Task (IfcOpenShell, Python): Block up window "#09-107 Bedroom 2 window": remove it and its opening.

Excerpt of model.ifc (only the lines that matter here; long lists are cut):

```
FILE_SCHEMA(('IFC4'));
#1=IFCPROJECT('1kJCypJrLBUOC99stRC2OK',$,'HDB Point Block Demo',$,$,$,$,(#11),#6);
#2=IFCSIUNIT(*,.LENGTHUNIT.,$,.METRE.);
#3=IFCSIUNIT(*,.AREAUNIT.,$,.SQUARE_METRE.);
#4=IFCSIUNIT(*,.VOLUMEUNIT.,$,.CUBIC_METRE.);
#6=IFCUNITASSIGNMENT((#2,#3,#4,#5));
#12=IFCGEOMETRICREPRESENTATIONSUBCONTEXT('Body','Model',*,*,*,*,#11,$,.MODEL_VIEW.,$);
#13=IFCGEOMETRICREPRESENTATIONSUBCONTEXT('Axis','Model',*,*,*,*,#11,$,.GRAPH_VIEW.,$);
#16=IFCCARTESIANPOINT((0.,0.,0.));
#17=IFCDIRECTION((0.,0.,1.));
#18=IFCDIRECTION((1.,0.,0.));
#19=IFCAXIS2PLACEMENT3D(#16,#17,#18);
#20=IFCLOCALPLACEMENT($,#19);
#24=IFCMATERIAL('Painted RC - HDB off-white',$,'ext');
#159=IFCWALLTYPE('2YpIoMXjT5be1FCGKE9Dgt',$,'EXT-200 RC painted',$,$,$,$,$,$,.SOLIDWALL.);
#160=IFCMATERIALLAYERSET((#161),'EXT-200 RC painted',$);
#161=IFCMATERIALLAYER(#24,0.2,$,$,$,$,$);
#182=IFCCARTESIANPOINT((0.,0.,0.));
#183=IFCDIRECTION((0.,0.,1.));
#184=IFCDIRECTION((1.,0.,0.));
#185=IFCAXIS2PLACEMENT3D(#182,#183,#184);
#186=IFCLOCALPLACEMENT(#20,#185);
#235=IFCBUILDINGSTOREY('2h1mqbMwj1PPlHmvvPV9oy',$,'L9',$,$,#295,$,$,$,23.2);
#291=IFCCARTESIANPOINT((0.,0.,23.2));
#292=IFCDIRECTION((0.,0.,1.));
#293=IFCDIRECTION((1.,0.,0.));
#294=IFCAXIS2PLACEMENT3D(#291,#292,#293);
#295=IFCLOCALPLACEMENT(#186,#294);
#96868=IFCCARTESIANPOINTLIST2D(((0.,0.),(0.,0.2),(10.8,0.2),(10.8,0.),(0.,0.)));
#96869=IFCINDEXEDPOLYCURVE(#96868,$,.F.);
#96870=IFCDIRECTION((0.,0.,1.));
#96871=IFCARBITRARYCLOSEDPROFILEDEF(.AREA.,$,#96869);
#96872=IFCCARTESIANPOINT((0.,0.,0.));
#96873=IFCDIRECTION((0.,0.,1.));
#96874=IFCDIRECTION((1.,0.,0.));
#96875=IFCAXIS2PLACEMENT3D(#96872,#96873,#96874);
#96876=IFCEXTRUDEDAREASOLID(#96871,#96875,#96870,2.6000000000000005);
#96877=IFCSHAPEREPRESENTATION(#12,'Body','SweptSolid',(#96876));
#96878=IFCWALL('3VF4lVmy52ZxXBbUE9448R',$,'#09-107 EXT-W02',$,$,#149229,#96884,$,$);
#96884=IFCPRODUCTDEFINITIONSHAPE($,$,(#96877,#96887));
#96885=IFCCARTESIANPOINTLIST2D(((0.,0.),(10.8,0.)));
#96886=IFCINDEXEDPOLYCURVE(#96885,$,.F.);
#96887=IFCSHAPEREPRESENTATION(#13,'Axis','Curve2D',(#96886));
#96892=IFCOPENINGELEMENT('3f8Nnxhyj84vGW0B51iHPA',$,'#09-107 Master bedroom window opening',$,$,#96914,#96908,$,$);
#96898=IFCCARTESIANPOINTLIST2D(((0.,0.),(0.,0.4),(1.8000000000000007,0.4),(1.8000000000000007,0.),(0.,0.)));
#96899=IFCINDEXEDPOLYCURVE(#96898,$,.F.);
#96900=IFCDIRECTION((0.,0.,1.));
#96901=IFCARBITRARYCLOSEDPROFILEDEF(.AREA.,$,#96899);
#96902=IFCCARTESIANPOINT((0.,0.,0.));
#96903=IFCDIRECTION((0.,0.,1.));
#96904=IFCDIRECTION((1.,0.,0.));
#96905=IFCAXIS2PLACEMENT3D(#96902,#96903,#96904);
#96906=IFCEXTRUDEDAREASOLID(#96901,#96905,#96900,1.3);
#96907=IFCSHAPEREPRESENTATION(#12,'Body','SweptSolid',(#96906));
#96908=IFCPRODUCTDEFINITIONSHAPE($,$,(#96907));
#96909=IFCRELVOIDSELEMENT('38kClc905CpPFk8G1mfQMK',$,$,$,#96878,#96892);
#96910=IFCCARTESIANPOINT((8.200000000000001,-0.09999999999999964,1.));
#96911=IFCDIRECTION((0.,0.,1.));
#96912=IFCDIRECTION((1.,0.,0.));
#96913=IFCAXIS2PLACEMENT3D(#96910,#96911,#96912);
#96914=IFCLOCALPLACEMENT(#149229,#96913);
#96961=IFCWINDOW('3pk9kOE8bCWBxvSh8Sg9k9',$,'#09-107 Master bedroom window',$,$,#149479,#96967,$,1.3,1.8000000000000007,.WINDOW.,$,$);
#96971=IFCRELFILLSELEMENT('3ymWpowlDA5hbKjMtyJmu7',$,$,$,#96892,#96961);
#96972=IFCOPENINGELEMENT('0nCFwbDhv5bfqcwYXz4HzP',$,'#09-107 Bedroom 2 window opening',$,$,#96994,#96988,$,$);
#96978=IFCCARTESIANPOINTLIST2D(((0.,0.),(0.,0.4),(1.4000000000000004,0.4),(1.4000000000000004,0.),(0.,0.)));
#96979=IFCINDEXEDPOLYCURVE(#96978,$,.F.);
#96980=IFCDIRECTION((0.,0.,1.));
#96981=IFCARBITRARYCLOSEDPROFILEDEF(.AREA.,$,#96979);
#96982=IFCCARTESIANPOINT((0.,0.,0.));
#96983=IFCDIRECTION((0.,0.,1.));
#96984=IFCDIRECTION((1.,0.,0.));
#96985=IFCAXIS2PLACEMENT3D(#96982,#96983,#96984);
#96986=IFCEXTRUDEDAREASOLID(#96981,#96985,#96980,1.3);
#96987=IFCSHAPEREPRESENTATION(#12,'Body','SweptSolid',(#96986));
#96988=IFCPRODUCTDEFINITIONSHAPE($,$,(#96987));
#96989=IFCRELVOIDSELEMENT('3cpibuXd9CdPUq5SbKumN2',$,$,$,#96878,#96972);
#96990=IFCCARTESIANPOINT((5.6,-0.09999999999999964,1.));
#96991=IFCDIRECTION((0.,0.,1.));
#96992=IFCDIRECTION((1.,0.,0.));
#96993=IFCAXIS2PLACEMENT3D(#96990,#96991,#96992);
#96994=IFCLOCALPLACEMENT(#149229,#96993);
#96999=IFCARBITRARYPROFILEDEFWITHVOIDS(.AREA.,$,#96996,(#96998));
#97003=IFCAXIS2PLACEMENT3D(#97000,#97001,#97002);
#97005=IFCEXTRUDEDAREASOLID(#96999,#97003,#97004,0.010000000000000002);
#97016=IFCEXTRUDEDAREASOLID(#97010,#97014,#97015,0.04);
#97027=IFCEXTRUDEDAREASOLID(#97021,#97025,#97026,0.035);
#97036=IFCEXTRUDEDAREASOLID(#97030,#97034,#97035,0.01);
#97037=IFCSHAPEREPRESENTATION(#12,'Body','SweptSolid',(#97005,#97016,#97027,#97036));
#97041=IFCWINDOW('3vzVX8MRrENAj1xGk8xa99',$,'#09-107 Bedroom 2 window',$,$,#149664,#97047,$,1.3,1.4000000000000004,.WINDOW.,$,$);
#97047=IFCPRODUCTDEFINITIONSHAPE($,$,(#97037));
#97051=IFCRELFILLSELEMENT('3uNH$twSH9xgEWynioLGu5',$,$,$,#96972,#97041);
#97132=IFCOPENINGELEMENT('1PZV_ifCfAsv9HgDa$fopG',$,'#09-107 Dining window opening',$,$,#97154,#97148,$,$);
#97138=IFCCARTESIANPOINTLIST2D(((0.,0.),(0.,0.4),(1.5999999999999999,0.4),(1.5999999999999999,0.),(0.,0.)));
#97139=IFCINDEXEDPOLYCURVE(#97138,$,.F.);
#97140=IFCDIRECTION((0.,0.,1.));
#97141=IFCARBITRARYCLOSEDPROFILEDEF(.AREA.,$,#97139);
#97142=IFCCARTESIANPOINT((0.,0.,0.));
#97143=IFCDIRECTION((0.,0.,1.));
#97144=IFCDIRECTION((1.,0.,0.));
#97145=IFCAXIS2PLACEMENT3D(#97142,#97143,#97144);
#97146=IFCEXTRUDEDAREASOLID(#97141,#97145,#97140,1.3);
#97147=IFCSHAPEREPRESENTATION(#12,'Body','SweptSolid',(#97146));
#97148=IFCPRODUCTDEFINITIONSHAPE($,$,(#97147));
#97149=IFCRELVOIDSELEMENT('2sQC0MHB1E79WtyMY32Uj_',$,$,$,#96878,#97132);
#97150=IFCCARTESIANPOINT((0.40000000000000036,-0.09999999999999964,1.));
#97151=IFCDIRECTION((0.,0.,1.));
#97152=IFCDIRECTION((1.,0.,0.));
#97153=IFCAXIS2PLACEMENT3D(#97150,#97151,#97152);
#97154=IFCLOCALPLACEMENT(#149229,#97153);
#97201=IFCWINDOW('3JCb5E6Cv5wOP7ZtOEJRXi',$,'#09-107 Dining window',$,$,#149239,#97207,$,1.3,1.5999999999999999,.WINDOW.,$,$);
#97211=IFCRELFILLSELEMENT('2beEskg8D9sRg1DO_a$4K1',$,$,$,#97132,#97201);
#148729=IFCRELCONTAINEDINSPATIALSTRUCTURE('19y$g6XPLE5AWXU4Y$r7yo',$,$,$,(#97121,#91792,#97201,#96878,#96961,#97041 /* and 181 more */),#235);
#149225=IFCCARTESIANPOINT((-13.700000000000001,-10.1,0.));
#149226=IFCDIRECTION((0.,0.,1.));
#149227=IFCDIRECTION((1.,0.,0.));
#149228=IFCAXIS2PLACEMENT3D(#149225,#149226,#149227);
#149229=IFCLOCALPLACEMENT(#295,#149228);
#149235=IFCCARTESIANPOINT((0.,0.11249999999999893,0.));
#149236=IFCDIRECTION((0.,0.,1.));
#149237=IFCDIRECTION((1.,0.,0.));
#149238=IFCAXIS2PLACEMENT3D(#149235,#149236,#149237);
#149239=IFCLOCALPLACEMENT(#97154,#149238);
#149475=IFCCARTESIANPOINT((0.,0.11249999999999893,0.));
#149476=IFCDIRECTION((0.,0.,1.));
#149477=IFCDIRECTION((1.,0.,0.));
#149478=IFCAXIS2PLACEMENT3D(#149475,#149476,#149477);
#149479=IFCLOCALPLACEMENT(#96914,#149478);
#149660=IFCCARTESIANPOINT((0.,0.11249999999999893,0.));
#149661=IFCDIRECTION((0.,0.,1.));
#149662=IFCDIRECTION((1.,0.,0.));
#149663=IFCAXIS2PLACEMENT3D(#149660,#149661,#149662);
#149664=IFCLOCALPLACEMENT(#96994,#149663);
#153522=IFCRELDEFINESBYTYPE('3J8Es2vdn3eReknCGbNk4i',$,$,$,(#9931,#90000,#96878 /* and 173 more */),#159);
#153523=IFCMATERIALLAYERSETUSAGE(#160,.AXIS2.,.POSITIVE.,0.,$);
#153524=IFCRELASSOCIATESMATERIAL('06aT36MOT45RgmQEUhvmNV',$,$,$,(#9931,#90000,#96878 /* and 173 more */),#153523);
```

```python
import ifcopenshell
import ifcopenshell.api.feature
import ifcopenshell.api.root
import ifcopenshell.geom
import ifcopenshell.util.shape

model = ifcopenshell.open("model.ifc")
settings = ifcopenshell.geom.settings()


def volume(element):
    """Net volume in cubic metres, openings subtracted."""
    shape = ifcopenshell.geom.create_shape(settings, element)
    return ifcopenshell.util.shape.get_volume(shape.geometry)


window = model.by_id(97041)
opening = window.FillsVoids[0].RelatingOpeningElement
wall = opening.VoidsElements[0].RelatingBuildingElement
before = volume(wall)

ifcopenshell.api.root.remove_product(model, product=window)
ifcopenshell.api.feature.remove_feature(model, feature=opening)

after = volume(wall)

print(f"wall volume {before:.3f} -> {after:.3f} m3")

model.write("model_rev.ifc")
```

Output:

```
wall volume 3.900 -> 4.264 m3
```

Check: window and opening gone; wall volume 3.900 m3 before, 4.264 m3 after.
